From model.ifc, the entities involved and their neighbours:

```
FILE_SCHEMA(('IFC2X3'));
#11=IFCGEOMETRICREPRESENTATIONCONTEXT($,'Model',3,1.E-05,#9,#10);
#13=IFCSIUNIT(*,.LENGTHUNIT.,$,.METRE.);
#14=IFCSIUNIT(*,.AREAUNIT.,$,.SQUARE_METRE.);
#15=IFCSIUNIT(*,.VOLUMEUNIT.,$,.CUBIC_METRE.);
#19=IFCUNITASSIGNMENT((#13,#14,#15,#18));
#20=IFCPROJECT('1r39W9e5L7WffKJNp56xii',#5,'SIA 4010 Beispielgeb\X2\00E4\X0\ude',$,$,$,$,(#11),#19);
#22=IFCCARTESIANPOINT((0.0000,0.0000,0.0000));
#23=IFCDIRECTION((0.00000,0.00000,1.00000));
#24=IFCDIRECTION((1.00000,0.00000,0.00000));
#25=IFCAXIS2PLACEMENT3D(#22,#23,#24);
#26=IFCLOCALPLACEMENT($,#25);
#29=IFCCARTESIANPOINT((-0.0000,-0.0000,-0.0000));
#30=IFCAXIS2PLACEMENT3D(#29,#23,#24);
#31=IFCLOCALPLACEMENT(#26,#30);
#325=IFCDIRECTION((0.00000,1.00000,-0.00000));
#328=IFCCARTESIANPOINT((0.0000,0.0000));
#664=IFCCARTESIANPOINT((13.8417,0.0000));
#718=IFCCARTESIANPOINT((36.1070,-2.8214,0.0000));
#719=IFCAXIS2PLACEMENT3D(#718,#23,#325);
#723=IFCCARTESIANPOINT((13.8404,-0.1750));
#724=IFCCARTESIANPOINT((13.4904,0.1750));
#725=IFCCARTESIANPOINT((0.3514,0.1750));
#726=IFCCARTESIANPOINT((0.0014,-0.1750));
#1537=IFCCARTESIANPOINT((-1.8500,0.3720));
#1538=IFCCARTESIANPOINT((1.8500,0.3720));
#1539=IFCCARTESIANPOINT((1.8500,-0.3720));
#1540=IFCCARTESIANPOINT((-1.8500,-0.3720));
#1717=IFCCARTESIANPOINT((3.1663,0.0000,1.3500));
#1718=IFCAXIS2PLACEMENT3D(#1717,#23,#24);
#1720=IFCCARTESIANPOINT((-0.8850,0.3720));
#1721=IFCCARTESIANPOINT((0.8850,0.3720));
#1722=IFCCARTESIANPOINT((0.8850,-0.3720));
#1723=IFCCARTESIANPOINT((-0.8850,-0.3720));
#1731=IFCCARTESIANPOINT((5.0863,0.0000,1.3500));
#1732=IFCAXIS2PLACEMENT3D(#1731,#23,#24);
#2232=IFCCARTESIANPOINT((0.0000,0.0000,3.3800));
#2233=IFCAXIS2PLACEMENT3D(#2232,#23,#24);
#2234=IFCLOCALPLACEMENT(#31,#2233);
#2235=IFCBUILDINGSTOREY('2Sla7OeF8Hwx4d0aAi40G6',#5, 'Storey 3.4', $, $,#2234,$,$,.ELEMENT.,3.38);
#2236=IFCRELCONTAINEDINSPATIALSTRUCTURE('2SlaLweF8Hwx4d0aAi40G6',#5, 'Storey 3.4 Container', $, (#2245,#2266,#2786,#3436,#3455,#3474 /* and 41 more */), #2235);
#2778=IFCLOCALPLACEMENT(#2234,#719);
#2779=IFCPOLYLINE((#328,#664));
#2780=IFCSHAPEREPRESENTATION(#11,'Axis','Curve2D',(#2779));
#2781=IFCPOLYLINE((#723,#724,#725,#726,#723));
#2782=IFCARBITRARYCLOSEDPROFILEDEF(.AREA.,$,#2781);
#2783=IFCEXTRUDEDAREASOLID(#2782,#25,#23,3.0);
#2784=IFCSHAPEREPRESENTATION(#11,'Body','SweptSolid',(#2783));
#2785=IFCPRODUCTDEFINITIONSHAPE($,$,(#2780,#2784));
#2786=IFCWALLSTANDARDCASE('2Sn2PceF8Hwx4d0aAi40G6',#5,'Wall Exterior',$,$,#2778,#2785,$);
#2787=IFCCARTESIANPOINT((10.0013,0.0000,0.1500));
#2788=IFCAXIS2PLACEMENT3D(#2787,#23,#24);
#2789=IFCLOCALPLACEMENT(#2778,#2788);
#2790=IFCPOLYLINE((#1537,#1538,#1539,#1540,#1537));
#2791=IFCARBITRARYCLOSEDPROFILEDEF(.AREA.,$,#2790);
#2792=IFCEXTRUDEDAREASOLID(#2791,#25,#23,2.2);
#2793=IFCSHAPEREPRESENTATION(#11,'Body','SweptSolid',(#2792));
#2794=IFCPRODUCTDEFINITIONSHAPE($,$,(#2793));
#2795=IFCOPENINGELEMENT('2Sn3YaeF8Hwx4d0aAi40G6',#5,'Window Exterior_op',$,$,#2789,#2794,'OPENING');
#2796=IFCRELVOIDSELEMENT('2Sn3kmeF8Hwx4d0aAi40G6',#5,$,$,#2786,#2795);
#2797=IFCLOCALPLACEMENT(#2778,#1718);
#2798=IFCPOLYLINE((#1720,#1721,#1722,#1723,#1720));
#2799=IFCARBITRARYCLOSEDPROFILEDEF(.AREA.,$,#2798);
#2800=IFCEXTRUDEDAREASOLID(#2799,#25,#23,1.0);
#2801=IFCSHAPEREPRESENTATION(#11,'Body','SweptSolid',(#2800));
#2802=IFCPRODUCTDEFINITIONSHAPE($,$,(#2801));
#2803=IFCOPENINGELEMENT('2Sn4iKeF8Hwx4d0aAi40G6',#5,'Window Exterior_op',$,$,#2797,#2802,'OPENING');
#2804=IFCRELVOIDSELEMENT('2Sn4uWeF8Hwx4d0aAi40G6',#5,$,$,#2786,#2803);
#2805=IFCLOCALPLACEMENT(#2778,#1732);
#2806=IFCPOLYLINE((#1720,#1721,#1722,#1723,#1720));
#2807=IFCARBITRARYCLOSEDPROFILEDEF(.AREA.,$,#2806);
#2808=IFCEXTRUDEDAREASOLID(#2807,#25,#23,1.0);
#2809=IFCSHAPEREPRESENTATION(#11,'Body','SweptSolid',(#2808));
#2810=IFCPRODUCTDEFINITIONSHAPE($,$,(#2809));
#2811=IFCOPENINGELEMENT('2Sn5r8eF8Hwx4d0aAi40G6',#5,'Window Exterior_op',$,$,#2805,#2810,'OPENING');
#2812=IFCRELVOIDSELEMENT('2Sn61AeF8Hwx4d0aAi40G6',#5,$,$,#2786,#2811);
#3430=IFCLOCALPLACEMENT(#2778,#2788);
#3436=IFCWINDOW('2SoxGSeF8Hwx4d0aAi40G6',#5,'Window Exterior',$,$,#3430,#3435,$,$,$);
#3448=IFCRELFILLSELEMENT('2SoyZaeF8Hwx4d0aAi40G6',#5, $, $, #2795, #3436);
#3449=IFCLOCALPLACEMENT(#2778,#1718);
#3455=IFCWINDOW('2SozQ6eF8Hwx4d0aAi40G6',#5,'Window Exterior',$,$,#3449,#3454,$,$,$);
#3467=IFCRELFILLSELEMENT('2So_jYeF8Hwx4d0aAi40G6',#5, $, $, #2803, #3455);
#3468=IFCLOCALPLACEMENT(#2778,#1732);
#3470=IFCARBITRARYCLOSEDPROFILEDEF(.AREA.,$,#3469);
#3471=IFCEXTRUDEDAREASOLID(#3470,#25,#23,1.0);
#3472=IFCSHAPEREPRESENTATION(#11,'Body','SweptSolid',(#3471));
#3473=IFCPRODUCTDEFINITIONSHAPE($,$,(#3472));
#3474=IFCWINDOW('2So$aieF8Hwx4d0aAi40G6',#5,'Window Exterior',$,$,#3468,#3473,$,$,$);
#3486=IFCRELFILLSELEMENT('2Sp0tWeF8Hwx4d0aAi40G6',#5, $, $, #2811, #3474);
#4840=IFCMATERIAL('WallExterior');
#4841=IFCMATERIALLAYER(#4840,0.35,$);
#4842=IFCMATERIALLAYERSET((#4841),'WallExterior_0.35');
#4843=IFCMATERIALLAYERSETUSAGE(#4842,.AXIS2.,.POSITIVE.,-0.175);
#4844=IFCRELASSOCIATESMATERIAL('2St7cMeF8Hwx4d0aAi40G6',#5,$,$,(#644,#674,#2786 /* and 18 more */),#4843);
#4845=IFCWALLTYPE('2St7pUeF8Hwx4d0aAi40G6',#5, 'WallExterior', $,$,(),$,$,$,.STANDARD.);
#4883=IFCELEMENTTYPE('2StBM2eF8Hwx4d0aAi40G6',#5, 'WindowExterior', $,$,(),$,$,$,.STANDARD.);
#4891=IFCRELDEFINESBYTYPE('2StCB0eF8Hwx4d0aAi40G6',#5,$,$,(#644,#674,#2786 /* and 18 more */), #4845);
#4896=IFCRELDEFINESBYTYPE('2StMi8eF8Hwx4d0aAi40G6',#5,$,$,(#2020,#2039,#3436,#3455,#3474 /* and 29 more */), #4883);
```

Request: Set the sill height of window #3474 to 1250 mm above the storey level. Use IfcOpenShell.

```python
import numpy as np
import ifcopenshell
import ifcopenshell.api.geometry
import ifcopenshell.geom
import ifcopenshell.util.element
import ifcopenshell.util.placement
import ifcopenshell.util.shape
import ifcopenshell.util.unit

model = ifcopenshell.open("model.ifc")
unit_scale = ifcopenshell.util.unit.calculate_unit_scale(model)

window = model.by_guid("2So$aieF8Hwx4d0aAi40G6")
opening = window.FillsVoids[0].RelatingOpeningElement
storey = ifcopenshell.util.element.get_container(window, ifc_class="IfcBuildingStorey")
level = ifcopenshell.util.placement.get_local_placement(storey.ObjectPlacement)[2, 3]

# The opening's origin need not be at the sill, so measure its lowest point.
shape = ifcopenshell.geom.create_shape(ifcopenshell.geom.settings(), opening)
bottom = ifcopenshell.util.shape.get_shape_bottom_elevation(shape, shape.geometry) / unit_scale
dz = level + 1.25 / unit_scale - bottom

shift = np.array([0.0, 0.0, dz])
# The window is not placed relative to its opening, so move both.
for product in (opening, window):
    matrix = ifcopenshell.util.placement.get_local_placement(product.ObjectPlacement)
    matrix[:3, 3] += shift
    ifcopenshell.api.geometry.edit_object_placement(model, product=product, matrix=matrix, is_si=False)

print(f"moved by {dz * unit_scale:+.3f} m")

model.write("model_updated.ifc")
```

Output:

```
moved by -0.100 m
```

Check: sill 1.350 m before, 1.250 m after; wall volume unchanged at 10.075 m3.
